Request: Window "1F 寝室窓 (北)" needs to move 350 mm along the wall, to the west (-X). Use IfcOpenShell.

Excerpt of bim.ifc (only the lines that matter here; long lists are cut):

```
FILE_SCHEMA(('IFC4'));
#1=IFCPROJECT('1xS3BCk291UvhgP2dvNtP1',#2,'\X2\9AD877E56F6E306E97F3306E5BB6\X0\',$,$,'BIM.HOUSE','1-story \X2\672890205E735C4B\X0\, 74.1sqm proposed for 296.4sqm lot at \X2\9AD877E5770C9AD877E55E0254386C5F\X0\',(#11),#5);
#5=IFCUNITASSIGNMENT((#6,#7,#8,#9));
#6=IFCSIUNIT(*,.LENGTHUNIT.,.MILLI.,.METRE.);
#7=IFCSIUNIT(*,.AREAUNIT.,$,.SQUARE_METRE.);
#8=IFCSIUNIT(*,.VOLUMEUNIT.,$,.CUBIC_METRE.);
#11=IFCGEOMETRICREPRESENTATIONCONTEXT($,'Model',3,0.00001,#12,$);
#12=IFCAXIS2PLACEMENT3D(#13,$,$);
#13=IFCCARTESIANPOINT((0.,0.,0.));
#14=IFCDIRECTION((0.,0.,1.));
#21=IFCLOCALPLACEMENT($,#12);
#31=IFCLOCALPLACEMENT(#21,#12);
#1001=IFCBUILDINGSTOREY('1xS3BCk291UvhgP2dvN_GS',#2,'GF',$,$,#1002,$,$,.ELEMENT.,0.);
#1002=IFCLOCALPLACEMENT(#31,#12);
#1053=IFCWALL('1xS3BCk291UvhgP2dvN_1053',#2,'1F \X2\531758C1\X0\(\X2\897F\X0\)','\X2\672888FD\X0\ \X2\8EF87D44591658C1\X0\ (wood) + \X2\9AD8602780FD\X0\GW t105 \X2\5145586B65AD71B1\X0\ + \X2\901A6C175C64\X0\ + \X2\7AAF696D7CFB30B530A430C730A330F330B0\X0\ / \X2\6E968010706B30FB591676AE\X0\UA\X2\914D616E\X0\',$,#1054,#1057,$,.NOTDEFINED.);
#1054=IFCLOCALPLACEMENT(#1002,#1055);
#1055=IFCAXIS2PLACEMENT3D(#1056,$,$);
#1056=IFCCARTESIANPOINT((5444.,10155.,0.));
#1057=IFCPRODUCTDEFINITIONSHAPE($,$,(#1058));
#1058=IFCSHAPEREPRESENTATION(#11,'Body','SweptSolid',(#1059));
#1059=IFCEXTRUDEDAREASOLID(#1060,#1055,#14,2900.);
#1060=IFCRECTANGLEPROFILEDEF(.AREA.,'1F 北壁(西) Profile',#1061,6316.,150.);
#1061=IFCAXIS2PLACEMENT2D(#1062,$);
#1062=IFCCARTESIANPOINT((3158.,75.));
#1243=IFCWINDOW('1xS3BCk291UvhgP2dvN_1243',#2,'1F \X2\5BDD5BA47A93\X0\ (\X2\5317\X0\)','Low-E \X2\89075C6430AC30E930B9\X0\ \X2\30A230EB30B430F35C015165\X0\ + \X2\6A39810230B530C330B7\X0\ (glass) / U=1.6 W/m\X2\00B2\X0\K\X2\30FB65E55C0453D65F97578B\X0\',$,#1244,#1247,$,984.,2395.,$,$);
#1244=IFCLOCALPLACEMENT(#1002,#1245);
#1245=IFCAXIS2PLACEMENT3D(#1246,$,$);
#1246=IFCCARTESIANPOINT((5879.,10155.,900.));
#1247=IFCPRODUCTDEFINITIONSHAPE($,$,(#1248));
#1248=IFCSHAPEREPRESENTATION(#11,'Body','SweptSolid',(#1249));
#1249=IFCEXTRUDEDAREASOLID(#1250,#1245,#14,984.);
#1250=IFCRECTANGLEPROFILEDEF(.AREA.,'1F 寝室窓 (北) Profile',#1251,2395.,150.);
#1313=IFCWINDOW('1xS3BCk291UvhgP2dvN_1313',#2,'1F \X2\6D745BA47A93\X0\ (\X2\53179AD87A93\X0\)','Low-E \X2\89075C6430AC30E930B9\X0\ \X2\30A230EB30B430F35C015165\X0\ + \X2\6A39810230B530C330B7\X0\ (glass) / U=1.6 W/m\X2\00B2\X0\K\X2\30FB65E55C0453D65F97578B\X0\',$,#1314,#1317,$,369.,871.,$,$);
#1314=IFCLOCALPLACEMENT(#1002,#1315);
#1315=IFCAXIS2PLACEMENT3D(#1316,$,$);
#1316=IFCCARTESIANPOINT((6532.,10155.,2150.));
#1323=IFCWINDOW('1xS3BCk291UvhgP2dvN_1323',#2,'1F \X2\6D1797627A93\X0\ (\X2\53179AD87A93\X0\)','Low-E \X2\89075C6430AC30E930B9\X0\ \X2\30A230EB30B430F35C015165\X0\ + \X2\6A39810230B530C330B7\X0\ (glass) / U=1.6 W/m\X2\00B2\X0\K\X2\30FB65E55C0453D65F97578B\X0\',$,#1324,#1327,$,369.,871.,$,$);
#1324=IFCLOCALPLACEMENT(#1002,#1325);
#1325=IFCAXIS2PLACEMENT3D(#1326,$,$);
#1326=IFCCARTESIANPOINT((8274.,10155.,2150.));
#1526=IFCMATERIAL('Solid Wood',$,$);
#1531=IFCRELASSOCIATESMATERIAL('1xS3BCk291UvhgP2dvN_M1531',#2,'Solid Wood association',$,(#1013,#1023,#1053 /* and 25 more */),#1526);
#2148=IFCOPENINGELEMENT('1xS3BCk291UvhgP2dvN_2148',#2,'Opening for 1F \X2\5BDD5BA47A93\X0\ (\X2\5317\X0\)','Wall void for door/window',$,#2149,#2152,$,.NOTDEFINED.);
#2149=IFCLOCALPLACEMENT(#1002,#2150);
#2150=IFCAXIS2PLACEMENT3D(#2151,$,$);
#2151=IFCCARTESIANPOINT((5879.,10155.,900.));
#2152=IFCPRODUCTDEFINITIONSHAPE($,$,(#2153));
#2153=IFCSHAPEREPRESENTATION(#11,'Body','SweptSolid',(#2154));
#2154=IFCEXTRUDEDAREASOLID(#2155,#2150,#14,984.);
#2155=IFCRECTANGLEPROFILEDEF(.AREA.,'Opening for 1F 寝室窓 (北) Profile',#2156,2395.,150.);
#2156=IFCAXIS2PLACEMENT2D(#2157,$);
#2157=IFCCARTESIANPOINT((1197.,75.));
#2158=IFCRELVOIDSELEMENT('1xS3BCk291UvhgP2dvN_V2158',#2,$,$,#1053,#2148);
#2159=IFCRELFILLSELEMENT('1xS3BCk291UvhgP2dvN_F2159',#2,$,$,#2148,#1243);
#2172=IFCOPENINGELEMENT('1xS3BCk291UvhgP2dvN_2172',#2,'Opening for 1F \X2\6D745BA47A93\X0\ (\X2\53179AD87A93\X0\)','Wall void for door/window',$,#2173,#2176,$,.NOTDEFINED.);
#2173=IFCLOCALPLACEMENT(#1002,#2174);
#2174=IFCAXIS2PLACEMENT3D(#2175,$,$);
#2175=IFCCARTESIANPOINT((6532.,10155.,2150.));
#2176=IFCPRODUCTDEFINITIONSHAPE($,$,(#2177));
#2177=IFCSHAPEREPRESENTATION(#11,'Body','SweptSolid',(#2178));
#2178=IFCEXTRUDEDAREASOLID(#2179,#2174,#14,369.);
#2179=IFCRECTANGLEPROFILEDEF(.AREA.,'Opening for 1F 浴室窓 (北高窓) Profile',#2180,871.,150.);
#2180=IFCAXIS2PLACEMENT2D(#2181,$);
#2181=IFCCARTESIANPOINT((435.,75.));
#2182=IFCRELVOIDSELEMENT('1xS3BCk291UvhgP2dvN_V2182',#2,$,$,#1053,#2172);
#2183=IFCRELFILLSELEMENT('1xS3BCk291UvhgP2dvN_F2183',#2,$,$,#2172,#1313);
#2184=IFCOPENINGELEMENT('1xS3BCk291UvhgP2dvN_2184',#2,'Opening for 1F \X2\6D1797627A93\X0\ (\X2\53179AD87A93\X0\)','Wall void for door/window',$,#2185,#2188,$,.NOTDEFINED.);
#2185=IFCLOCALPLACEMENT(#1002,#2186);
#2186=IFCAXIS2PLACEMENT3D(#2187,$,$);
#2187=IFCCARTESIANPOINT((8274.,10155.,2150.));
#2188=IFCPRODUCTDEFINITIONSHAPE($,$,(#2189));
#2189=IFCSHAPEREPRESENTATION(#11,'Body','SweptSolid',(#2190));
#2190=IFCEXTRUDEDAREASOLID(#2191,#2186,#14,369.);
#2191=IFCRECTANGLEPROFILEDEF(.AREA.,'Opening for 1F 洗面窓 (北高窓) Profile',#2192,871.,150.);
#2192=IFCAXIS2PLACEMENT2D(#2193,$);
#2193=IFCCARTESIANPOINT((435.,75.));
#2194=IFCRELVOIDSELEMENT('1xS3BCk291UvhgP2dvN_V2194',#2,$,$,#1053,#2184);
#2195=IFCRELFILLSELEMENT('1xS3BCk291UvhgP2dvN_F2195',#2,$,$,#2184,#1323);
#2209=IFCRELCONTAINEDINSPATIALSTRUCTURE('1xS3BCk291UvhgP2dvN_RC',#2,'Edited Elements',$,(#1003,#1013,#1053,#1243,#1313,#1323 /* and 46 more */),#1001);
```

```python
import ifcopenshell
import ifcopenshell.api.geometry
import ifcopenshell.util.placement

model = ifcopenshell.open("bim.ifc")

window = model.by_guid("1xS3BCk291UvhgP2dvN_1243")
opening = window.FillsVoids[0].RelatingOpeningElement
wall = opening.VoidsElements[0].RelatingBuildingElement

wall_matrix = ifcopenshell.util.placement.get_local_placement(wall.ObjectPlacement)
shift = wall_matrix[:3, 0] * -350.0
before = ifcopenshell.util.placement.get_local_placement(window.ObjectPlacement)[:3, 3].copy()

# The window is not placed relative to its opening, so move both.
for product in (opening, window):
    matrix = ifcopenshell.util.placement.get_local_placement(product.ObjectPlacement)
    matrix[:3, 3] += shift
    ifcopenshell.api.geometry.edit_object_placement(model, product=product, matrix=matrix, is_si=False)

after = ifcopenshell.util.placement.get_local_placement(window.ObjectPlacement)[:3, 3]
print("window moved by", (after - before).round(3) + 0.0)

model.write("bim_edited.ifc")
```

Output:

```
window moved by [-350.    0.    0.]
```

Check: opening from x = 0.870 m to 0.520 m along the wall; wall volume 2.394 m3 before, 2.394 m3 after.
